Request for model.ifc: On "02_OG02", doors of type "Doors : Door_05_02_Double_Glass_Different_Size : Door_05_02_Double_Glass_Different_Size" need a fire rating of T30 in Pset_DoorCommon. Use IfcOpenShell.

First a look at what the model holds.

```python
import ifcopenshell
import ifcopenshell.util.element

model = ifcopenshell.open("model.ifc")
print(model.schema)
storey = next(s for s in model.by_type("IfcBuildingStorey") if s.Name == "02_OG02")
doors = [e for e in ifcopenshell.util.element.get_decomposition(storey) if e.is_a("IfcDoor")]
seen = {}
for e in doors:
    element_type = ifcopenshell.util.element.get_type(e)
    key = (element_type.Name if element_type != e and element_type else None, ifcopenshell.util.element.get_pset(e, "Pset_DoorCommon", "FireRating"))
    seen[key] = seen.get(key, 0) + 1
for (name, value), count in sorted(seen.items(), key=str):
    print(count, "x", name, "|", value)
```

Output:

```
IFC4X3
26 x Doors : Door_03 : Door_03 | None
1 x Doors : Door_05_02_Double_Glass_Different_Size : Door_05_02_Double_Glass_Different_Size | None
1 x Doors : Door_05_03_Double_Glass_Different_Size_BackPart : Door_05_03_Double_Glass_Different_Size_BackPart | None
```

```python
import ifcopenshell
import ifcopenshell.api.pset
import ifcopenshell.util.element

model = ifcopenshell.open("model.ifc")

storey = next(s for s in model.by_type("IfcBuildingStorey") if s.Name == "02_OG02")
doors = [e for e in ifcopenshell.util.element.get_decomposition(storey) if e.is_a("IfcDoor")]

count = 0
for e in doors:
    element_type = ifcopenshell.util.element.get_type(e)
    if element_type in (None, e) or element_type.Name != "Doors : Door_05_02_Double_Glass_Different_Size : Door_05_02_Double_Glass_Different_Size":
        continue
    # add_pset returns the element's existing set when there is one.
    pset = ifcopenshell.api.pset.add_pset(model, product=e, name="Pset_DoorCommon")
    ifcopenshell.api.pset.edit_pset(model, pset=pset, properties={"FireRating": "T30"})
    count += 1

print(count, "doors updated")

model.write("model_rev.ifc")
```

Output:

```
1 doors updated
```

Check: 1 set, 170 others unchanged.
